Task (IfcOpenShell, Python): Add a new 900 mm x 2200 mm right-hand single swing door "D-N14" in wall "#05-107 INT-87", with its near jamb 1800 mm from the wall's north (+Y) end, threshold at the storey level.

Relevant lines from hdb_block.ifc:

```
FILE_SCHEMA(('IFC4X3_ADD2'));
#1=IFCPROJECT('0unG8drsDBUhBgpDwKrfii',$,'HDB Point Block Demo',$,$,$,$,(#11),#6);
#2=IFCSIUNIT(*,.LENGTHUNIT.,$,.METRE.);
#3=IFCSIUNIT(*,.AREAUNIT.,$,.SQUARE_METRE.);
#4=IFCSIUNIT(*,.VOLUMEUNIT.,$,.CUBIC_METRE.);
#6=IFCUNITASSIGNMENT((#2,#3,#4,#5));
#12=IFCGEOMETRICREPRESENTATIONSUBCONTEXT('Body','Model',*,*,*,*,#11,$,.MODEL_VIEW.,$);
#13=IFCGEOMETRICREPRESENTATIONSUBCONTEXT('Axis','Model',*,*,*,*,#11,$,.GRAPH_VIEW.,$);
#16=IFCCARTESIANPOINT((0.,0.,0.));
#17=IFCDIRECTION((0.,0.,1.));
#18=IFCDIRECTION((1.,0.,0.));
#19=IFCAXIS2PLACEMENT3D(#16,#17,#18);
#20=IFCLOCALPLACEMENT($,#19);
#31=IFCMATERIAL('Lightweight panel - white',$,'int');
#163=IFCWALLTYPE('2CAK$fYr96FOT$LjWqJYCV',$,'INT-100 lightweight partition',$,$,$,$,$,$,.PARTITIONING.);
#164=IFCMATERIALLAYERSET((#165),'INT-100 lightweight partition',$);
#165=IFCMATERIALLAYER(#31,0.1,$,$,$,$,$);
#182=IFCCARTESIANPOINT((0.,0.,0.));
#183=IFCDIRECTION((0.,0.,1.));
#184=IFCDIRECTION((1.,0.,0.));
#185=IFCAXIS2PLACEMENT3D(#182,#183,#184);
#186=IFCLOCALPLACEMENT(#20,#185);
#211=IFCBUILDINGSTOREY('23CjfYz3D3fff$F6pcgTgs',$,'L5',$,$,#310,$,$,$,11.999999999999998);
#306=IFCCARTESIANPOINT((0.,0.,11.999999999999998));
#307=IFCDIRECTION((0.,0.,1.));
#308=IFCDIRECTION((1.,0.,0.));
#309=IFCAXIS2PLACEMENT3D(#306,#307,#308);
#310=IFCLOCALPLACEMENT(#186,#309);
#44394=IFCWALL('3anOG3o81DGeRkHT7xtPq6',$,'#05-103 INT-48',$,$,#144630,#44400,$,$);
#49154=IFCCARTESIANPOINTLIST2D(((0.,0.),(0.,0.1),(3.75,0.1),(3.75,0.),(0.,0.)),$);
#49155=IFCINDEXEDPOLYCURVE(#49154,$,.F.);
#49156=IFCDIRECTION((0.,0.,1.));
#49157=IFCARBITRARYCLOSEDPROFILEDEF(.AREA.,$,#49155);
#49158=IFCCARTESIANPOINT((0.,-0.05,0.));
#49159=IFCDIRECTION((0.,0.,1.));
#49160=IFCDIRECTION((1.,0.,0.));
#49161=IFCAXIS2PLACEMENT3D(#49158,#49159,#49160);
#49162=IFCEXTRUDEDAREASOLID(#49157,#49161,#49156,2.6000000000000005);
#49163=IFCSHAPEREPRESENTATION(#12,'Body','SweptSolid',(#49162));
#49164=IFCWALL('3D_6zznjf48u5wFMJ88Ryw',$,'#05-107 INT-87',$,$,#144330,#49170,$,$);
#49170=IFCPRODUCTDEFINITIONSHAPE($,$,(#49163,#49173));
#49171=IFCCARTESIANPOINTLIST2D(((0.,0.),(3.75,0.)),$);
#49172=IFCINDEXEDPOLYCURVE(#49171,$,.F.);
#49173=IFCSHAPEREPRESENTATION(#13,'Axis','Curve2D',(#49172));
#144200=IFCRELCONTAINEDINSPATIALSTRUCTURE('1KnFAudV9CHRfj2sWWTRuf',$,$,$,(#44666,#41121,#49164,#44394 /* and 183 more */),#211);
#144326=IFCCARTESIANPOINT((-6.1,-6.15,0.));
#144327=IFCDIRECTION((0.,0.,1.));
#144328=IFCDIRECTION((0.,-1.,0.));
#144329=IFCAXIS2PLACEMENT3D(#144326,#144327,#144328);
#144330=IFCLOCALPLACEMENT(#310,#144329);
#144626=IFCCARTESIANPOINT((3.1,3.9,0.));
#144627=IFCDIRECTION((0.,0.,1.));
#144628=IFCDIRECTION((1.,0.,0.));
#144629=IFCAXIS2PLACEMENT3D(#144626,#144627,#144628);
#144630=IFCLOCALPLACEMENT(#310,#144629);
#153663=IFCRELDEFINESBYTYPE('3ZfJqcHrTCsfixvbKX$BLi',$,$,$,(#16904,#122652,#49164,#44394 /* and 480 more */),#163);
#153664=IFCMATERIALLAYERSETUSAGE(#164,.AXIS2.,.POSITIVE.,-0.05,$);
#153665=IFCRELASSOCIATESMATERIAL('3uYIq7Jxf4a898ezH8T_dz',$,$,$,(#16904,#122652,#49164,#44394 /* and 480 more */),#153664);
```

```python
import numpy as np
import ifcopenshell
import ifcopenshell.api.feature
import ifcopenshell.api.geometry
import ifcopenshell.api.root
import ifcopenshell.api.spatial
import ifcopenshell.geom
import ifcopenshell.util.element
import ifcopenshell.util.placement
import ifcopenshell.util.representation
import ifcopenshell.util.shape
import ifcopenshell.util.unit

model = ifcopenshell.open("hdb_block.ifc")
unit_scale = ifcopenshell.util.unit.calculate_unit_scale(model)
settings = ifcopenshell.geom.settings()


def volume(element):
    """Net volume in cubic metres, openings subtracted."""
    shape = ifcopenshell.geom.create_shape(settings, element)
    return ifcopenshell.util.shape.get_volume(shape.geometry)


wall = model.by_guid("3D_6zznjf48u5wFMJ88Ryw")
storey = ifcopenshell.util.element.get_container(wall, ifc_class="IfcBuildingStorey")
context = ifcopenshell.util.representation.get_context(model, "Model", "Body", "MODEL_VIEW")
before = volume(wall)

width, height, from_end, sill = 0.9, 2.2, 1.8, 0.0  # metres

# The wall runs along its own X axis, and the end named is its -X end.
wall_shape = ifcopenshell.geom.create_shape(settings, wall)
x, y, z = ifcopenshell.util.shape.get_vertices(wall_shape.geometry).T
start = x.min() + from_end
face, thickness = float(y.min()), float(y.max() - y.min())
wall_matrix = ifcopenshell.util.placement.get_local_placement(wall.ObjectPlacement)
level = ifcopenshell.util.placement.get_local_placement(storey.ObjectPlacement)[2, 3]


def in_wall(x, y):
    """Placement at x, y metres in the wall's axes, at sill height."""
    matrix = wall_matrix.copy()
    matrix[:, 3] = wall_matrix @ np.array([x / unit_scale, y / unit_scale, 0.0, 1.0])
    matrix[2, 3] = level + sill / unit_scale
    return matrix


# Opening: a box that overshoots both wall faces by 50 mm.
opening = ifcopenshell.api.root.create_entity(model, ifc_class="IfcOpeningElement", predefined_type="OPENING")
box = ifcopenshell.api.geometry.add_wall_representation(
    model, context=context, length=width, height=height, thickness=thickness + 0.1
)
ifcopenshell.api.geometry.assign_representation(model, product=opening, representation=box)
ifcopenshell.api.geometry.edit_object_placement(model, product=opening, matrix=in_wall(start, face - 0.05), is_si=False)
ifcopenshell.api.feature.add_feature(model, feature=opening, element=wall)

door = ifcopenshell.api.root.create_entity(model, ifc_class="IfcDoor", name="D-N14", predefined_type="DOOR")
door.OverallWidth, door.OverallHeight = width / unit_scale, height / unit_scale
door.OperationType = "SINGLE_SWING_RIGHT"
body = ifcopenshell.api.geometry.add_door_representation(
    model,
    context=context,
    overall_width=door.OverallWidth,
    overall_height=door.OverallHeight,
    operation_type="SINGLE_SWING_RIGHT",
    lining_properties={"LiningDepth": thickness / unit_scale, "ThresholdDepth": thickness / unit_scale},
)
ifcopenshell.api.geometry.assign_representation(model, product=door, representation=body)
ifcopenshell.api.spatial.assign_container(model, products=[door], relating_structure=storey)
ifcopenshell.api.feature.add_filling(model, opening=opening, element=door)

# The lining spans the wall, so the door starts at the wall face.
ifcopenshell.api.geometry.edit_object_placement(model, product=door, matrix=in_wall(start, face), is_si=False)

after = volume(wall)

print(f"wall volume {before:.3f} -> {after:.3f} m3")

model.write("hdb_block_updated.ifc")
```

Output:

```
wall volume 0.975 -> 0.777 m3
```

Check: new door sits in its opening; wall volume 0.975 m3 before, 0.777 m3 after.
